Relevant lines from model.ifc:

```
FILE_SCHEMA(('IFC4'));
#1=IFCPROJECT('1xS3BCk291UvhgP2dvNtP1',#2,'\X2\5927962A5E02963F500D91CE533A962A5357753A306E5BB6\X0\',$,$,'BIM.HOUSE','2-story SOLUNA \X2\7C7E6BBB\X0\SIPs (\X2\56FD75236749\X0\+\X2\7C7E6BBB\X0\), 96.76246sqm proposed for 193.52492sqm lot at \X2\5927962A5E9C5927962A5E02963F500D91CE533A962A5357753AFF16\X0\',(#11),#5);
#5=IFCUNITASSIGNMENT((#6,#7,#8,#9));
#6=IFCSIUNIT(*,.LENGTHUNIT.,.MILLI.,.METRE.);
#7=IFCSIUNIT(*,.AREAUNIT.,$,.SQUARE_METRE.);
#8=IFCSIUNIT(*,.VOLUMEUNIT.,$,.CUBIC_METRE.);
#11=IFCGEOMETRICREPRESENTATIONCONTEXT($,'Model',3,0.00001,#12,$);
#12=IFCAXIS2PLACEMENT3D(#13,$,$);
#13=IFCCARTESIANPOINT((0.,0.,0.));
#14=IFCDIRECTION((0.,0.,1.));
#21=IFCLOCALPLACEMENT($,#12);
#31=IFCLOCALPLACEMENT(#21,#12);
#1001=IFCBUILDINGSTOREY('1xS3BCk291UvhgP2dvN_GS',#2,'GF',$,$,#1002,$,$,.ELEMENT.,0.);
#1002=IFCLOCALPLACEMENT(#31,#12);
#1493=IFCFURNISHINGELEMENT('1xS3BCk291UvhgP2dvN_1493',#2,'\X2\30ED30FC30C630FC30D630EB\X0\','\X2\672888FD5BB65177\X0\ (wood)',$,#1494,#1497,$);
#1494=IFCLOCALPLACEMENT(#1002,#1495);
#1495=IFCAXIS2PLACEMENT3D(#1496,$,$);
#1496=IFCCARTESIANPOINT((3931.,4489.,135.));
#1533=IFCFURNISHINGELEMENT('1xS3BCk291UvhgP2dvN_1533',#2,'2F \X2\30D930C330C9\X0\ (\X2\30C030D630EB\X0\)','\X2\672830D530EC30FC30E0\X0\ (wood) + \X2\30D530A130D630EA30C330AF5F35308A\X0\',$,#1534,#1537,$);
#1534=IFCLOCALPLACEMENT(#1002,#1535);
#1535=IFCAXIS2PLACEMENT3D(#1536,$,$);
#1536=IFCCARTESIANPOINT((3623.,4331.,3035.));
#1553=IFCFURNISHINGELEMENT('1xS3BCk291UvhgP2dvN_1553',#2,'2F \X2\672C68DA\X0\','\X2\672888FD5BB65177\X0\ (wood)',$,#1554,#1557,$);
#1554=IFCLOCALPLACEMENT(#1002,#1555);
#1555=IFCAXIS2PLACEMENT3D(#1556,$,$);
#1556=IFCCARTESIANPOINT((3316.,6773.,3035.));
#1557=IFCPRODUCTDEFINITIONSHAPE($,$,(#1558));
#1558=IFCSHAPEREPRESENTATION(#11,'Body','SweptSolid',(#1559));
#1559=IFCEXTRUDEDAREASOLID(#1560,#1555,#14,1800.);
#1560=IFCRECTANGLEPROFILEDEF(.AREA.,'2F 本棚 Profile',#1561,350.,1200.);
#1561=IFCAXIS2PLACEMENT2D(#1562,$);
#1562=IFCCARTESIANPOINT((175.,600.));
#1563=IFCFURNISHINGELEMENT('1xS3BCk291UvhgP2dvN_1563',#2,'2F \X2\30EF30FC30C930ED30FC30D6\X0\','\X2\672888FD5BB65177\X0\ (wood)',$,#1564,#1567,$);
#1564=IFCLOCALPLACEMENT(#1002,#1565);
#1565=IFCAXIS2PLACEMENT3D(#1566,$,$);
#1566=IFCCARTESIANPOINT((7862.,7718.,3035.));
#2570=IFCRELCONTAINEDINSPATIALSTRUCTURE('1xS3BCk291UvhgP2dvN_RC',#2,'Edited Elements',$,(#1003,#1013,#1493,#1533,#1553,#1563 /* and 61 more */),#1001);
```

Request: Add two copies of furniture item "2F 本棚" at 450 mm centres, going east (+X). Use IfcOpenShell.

```python
import numpy as np
import ifcopenshell
import ifcopenshell.api.geometry
import ifcopenshell.api.root
import ifcopenshell.util.element
import ifcopenshell.util.placement

model = ifcopenshell.open("model.ifc")


def reuse_history(source, copy):
    """copy_class also copies each property set's owner history, people and application; keep the originals."""
    for rel in copy.IsDefinedBy:
        if rel.is_a("IfcRelDefinesByProperties") and (history := rel.RelatingPropertyDefinition.OwnerHistory):
            rel.RelatingPropertyDefinition.OwnerHistory = source.OwnerHistory
            ifcopenshell.util.element.remove_deep2(model, history)


source = model.by_guid("1xS3BCk291UvhgP2dvN_1553")
base = ifcopenshell.util.placement.get_local_placement(source.ObjectPlacement)
step = np.array([1.0, 0.0, 0.0]) * 450.0

for i in range(1, 3):
    copy = ifcopenshell.api.root.copy_class(model, product=source)
    copy.Representation = ifcopenshell.util.element.copy_deep(
        model, source.Representation, exclude=["IfcGeometricRepresentationContext", "IfcRepresentationMap"]
    )
    reuse_history(source, copy)
    matrix = base.copy()
    matrix[:3, 3] += i * step
    print("added at", matrix[:3, 3].round(3) + 0.0)
    ifcopenshell.api.geometry.edit_object_placement(model, product=copy, matrix=matrix, is_si=False)

model.write("model_v2.ifc")
```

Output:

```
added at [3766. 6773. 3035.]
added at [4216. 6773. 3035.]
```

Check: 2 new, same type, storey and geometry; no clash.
